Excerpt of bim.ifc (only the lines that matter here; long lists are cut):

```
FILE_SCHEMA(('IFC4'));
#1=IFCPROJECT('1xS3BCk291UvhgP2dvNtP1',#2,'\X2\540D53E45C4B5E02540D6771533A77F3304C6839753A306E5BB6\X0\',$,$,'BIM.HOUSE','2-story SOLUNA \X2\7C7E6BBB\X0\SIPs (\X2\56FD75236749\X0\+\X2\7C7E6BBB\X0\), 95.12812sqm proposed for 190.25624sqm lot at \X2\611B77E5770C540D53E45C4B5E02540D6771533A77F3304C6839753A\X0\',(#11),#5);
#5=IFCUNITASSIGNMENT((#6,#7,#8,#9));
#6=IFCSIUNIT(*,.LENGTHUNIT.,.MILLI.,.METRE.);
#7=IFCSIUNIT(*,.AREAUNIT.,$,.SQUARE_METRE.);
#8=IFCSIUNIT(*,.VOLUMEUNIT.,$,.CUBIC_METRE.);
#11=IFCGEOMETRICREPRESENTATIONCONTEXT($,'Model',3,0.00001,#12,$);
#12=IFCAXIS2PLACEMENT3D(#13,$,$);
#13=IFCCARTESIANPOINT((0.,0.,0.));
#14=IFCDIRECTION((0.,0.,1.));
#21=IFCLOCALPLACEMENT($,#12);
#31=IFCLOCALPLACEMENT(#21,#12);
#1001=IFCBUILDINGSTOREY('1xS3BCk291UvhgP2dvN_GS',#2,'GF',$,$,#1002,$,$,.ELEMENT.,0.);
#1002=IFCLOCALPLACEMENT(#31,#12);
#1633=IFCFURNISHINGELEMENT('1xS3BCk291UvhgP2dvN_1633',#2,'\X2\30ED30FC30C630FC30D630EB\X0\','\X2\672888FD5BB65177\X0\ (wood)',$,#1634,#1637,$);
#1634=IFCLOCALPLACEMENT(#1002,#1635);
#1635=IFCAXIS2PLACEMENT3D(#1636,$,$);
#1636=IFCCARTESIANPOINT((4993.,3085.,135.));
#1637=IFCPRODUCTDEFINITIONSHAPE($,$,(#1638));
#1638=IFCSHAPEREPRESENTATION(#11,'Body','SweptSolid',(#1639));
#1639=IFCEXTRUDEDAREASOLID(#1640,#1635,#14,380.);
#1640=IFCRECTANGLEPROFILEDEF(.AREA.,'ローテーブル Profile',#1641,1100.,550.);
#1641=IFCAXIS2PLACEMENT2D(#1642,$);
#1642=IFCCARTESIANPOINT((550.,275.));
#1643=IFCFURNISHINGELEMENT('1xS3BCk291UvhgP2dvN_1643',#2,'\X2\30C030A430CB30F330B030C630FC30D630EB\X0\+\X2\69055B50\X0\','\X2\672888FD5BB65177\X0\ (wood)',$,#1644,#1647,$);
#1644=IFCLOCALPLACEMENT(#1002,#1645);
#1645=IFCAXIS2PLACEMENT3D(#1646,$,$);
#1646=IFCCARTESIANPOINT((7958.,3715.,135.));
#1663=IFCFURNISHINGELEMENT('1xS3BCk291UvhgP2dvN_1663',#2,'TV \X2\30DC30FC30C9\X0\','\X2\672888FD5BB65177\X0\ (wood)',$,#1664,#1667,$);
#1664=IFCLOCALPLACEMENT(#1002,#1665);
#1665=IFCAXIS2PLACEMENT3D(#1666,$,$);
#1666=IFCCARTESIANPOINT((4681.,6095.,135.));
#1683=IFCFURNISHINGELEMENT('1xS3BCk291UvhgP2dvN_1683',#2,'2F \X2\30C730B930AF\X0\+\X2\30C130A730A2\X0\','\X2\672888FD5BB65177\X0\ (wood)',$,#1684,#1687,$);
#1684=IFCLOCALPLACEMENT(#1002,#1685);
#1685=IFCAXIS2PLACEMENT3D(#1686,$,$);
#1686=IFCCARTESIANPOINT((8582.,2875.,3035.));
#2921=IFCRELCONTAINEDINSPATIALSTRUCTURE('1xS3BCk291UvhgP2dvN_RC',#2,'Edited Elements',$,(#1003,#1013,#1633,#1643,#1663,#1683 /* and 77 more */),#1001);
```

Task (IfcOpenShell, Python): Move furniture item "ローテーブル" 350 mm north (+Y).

```python
import ifcopenshell
import ifcopenshell.api.geometry
import ifcopenshell.util.placement

model = ifcopenshell.open("bim.ifc")

item = model.by_id(1633)
matrix = ifcopenshell.util.placement.get_local_placement(item.ObjectPlacement)
matrix[1, 3] += 350.0
ifcopenshell.api.geometry.edit_object_placement(model, product=item, matrix=matrix, is_si=False)

print(ifcopenshell.util.placement.get_local_placement(item.ObjectPlacement).round(3) + 0.0)

model.write("bim-out.ifc")
```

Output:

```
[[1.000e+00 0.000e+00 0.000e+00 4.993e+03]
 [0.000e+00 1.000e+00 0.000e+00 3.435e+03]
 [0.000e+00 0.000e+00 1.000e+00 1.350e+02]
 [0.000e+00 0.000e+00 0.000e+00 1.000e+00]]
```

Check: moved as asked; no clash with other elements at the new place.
